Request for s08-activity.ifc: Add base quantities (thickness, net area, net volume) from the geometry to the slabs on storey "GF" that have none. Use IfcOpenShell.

First a look at what the model holds.

```python
import ifcopenshell
import ifcopenshell.util.element
import ifcopenshell.util.unit

model = ifcopenshell.open("s08-activity.ifc")
print(model.schema)
for unit_type in ("LENGTHUNIT", "AREAUNIT", "VOLUMEUNIT"):
    print(unit_type, ifcopenshell.util.unit.calculate_unit_scale(model, unit_type))
storey = next(s for s in model.by_type("IfcBuildingStorey") if s.Name == "GF")
slabs = [e for e in ifcopenshell.util.element.get_decomposition(storey) if e.is_a("IfcSlab")]
for e in sorted(slabs, key=lambda e: e.id()):
    print(e.id(), e.is_a(), e.Name, list(ifcopenshell.util.element.get_psets(e, qtos_only=True)), sep=" | ")
```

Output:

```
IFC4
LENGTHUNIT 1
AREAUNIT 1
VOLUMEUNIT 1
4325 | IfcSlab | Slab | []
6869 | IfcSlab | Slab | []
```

```python
import ifcopenshell
import ifcopenshell.api.pset
import ifcopenshell.geom
import ifcopenshell.util.element
import ifcopenshell.util.shape
import ifcopenshell.util.unit

model = ifcopenshell.open("s08-activity.ifc")
unit_scale = ifcopenshell.util.unit.calculate_unit_scale(model)
area_scale = ifcopenshell.util.unit.calculate_unit_scale(model, "AREAUNIT")
volume_scale = ifcopenshell.util.unit.calculate_unit_scale(model, "VOLUMEUNIT")
settings = ifcopenshell.geom.settings()

storey = next(s for s in model.by_type("IfcBuildingStorey") if s.Name == "GF")
slabs = [e for e in ifcopenshell.util.element.get_decomposition(storey) if e.is_a("IfcSlab")]

for e in sorted(slabs, key=lambda e: e.id()):
    if ifcopenshell.util.element.get_psets(e, qtos_only=True, should_inherit=False):
        continue
    # Geometry comes back in metres, in the element's own axes.
    shape = ifcopenshell.geom.create_shape(settings, e)
    values = {
        "Width": ifcopenshell.util.shape.get_z(shape.geometry) / unit_scale,
        "NetArea": ifcopenshell.util.shape.get_footprint_area(shape.geometry) / area_scale,
        "NetVolume": ifcopenshell.util.shape.get_volume(shape.geometry) / volume_scale,
    }
    qto = ifcopenshell.api.pset.add_qto(model, product=e, name="Qto_SlabBaseQuantities")
    ifcopenshell.api.pset.edit_qto(model, qto=qto, properties=values)
    print(e.id(), {k: round(v, 3) for k, v in values.items()})

model.write("s08-activity_edited.ifc")
```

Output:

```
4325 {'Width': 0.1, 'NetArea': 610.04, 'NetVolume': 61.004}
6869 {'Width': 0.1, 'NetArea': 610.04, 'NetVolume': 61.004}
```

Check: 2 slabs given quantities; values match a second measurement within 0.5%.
